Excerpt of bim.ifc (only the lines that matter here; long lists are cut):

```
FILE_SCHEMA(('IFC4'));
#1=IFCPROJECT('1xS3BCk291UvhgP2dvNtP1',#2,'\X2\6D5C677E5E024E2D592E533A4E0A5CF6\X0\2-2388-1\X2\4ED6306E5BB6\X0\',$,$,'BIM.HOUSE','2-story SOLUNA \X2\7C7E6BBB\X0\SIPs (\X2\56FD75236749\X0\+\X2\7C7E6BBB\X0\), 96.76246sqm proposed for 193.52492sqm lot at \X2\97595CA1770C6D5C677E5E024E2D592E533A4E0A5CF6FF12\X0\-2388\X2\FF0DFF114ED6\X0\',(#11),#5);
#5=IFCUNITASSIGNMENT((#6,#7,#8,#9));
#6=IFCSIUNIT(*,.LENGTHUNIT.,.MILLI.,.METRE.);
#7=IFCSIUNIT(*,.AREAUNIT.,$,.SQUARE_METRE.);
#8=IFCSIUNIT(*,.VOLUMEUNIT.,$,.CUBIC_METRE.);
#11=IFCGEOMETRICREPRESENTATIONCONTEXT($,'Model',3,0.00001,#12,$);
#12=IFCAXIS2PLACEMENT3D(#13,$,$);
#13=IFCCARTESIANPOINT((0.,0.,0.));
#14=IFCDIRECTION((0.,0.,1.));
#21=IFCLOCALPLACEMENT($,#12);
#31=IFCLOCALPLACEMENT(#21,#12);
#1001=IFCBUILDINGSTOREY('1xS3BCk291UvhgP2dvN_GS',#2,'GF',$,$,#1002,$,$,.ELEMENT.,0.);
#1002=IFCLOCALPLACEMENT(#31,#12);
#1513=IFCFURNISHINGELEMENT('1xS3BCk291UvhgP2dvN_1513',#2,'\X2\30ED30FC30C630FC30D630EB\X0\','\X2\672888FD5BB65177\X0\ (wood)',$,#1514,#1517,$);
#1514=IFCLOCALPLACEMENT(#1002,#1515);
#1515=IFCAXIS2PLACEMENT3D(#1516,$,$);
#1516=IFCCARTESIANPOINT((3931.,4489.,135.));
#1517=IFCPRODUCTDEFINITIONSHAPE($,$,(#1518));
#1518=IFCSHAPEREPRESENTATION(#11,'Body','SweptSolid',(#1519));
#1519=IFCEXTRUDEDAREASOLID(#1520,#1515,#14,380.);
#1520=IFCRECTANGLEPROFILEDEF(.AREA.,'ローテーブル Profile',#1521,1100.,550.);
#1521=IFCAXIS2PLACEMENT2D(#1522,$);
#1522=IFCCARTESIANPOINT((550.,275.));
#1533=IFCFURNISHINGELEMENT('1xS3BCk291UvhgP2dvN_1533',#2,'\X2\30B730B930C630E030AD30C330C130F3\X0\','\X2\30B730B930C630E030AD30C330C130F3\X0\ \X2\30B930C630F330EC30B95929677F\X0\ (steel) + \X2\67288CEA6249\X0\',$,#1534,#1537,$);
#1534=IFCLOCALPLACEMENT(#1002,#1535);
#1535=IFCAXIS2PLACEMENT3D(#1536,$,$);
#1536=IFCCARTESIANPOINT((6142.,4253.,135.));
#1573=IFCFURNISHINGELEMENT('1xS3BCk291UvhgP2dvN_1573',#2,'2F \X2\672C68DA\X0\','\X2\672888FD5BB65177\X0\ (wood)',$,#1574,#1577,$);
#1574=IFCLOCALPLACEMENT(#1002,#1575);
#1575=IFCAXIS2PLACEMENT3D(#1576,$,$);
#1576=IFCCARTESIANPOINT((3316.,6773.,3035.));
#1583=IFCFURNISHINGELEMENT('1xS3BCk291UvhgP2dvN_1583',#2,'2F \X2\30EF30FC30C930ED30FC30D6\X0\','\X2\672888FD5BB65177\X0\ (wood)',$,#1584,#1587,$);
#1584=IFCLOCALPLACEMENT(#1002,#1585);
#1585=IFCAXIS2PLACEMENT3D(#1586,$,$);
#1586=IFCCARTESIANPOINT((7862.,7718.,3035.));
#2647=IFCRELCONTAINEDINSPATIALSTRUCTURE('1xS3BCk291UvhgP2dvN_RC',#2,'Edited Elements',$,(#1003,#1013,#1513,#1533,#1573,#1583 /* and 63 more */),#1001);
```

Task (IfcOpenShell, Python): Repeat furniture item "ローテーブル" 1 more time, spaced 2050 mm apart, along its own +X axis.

```python
import ifcopenshell
import ifcopenshell.api.geometry
import ifcopenshell.api.root
import ifcopenshell.util.element
import ifcopenshell.util.placement
import ifcopenshell.util.unit

model = ifcopenshell.open("bim.ifc")
unit_scale = ifcopenshell.util.unit.calculate_unit_scale(model)


def reuse_history(source, copy):
    """copy_class also copies each property set's owner history, people and application; keep the originals."""
    for rel in copy.IsDefinedBy:
        if rel.is_a("IfcRelDefinesByProperties") and (history := rel.RelatingPropertyDefinition.OwnerHistory):
            rel.RelatingPropertyDefinition.OwnerHistory = source.OwnerHistory
            ifcopenshell.util.element.remove_deep2(model, history)


source = model.by_guid("1xS3BCk291UvhgP2dvN_1513")
base = ifcopenshell.util.placement.get_local_placement(source.ObjectPlacement)
step = base[:3, 0] * 2.05 / unit_scale

for i in range(1, 2):
    copy = ifcopenshell.api.root.copy_class(model, product=source)
    copy.Representation = ifcopenshell.util.element.copy_deep(
        model, source.Representation, exclude=["IfcGeometricRepresentationContext", "IfcRepresentationMap"]
    )
    reuse_history(source, copy)
    matrix = base.copy()
    matrix[:3, 3] += i * step
    print("added at", matrix[:3, 3].round(3) + 0.0)
    ifcopenshell.api.geometry.edit_object_placement(model, product=copy, matrix=matrix, is_si=False)

model.write("bim_edited.ifc")
```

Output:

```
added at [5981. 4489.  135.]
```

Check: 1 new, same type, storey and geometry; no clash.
